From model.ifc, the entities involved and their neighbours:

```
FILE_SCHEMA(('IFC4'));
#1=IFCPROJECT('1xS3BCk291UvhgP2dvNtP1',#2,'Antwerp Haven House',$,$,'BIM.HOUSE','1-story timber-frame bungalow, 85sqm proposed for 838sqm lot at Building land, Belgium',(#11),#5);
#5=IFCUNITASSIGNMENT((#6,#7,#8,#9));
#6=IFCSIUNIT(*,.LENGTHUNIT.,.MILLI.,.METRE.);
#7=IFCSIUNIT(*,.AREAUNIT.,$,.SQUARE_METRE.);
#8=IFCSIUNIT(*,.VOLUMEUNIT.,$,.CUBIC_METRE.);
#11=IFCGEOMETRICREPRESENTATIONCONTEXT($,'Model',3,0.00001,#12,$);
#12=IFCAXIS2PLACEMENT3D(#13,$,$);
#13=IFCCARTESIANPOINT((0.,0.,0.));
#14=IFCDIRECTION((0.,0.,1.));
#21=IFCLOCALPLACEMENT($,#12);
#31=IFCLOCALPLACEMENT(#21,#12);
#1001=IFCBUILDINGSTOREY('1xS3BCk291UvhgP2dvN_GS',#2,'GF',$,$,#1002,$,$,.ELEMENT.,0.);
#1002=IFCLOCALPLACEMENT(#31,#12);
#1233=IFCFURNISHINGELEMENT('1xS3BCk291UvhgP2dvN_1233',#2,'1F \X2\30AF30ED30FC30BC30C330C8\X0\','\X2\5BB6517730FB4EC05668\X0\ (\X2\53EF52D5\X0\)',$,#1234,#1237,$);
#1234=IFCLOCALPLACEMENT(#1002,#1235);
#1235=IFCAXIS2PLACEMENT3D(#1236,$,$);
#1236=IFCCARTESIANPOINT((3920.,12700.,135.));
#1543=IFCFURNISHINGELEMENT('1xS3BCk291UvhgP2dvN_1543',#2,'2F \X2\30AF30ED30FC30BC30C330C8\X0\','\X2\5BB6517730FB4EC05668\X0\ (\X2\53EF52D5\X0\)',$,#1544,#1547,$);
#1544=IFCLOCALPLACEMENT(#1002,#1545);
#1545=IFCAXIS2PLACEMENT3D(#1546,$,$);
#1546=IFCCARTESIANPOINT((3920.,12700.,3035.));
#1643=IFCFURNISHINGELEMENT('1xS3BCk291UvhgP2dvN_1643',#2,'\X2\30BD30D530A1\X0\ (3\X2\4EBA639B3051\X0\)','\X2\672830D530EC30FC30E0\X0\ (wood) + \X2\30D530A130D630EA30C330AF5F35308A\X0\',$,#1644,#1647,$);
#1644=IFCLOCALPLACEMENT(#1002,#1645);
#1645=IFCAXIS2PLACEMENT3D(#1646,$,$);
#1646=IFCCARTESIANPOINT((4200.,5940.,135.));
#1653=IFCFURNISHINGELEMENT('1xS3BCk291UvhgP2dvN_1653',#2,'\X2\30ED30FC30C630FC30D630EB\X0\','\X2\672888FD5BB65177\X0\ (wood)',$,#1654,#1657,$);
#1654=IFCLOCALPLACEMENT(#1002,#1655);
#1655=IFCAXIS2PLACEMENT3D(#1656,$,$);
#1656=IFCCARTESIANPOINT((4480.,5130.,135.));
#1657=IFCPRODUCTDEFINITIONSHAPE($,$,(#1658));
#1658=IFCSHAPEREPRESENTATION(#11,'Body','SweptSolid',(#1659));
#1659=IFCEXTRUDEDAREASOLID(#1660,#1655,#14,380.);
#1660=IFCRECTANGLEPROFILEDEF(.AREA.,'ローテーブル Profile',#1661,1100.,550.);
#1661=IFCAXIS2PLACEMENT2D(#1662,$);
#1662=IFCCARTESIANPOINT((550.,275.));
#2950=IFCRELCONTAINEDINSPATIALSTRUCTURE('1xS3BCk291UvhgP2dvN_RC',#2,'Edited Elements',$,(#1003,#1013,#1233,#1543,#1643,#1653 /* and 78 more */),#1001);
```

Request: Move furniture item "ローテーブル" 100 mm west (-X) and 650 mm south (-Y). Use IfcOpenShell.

```python
import ifcopenshell
import ifcopenshell.api.geometry
import ifcopenshell.util.placement

model = ifcopenshell.open("model.ifc")

item = model.by_guid("1xS3BCk291UvhgP2dvN_1653")
matrix = ifcopenshell.util.placement.get_local_placement(item.ObjectPlacement)
matrix[0, 3] -= 100.0
matrix[1, 3] -= 650.0
ifcopenshell.api.geometry.edit_object_placement(model, product=item, matrix=matrix, is_si=False)

print(ifcopenshell.util.placement.get_local_placement(item.ObjectPlacement).round(3) + 0.0)

model.write("model_updated.ifc")
```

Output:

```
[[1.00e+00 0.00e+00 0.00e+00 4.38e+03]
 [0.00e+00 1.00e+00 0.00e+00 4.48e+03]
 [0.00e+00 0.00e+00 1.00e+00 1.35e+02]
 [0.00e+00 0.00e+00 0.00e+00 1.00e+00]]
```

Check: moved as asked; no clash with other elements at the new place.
